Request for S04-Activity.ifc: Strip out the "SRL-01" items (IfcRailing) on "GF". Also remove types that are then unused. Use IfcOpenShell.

First a look at what the model holds.

```python
import ifcopenshell
import ifcopenshell.util.element

model = ifcopenshell.open("S04-Activity.ifc")
print(model.schema)
storey = next(s for s in model.by_type("IfcBuildingStorey") if s.Name == "GF")
railings = [e for e in ifcopenshell.util.element.get_decomposition(storey) if e.is_a("IfcRailing")]
seen = {}
for e in railings:
    element_type = ifcopenshell.util.element.get_type(e)
    name = element_type.Name if element_type not in (None, e) else None
    seen[name] = seen.get(name, 0) + 1
for name, count in sorted(seen.items(), key=str):
    print(count, "x", name)
```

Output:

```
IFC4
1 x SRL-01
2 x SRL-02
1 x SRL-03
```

```python
import ifcopenshell
import ifcopenshell.api.root
import ifcopenshell.util.element

model = ifcopenshell.open("S04-Activity.ifc")

storey = next(s for s in model.by_type("IfcBuildingStorey") if s.Name == "GF")
railings = [e for e in ifcopenshell.util.element.get_decomposition(storey) if e.is_a("IfcRailing")]
targets = [e for e in railings if (t := ifcopenshell.util.element.get_type(e)) not in (None, e) and t.Name == "SRL-01"]
types = {ifcopenshell.util.element.get_type(e) for e in targets} - {None, *targets}

for e in targets:
    ifcopenshell.api.root.remove_product(model, product=e)
print(len(targets), "removed")

unused = [t for t in types if not ifcopenshell.util.element.get_types(t)]
for t in unused:
    ifcopenshell.api.root.remove_product(model, product=t)
print(len(unused), "unused types removed")

model.write("S04-Activity_updated.ifc")
```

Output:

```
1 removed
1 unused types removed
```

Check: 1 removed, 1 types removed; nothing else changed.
